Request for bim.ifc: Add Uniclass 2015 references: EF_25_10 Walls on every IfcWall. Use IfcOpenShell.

First a look at what the model holds.

```python
import ifcopenshell

model = ifcopenshell.open("bim.ifc")
print(model.schema)
print("classifications:", [c.Name for c in model.by_type("IfcClassification")])
for ifc_class in ("IfcDoor", "IfcRoof", "IfcStair", "IfcWall", "IfcWindow"):
    print(ifc_class, len(model.by_type(ifc_class)))
```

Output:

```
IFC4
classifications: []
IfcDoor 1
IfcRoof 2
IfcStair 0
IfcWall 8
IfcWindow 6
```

```python
import ifcopenshell
import ifcopenshell.api.classification

model = ifcopenshell.open("bim.ifc")

system = ifcopenshell.api.classification.add_classification(model, classification="Uniclass 2015")

codes = {
    "IfcWall": ("EF_25_10", "Walls"),
}
for ifc_class, (code, name) in codes.items():
    products = model.by_type(ifc_class)
    ifcopenshell.api.classification.add_reference(
        model, products=products, classification=system, identification=code, name=name
    )
    print(code, len(products))

model.write("bim_rev.ifc")
```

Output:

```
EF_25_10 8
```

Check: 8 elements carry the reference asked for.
